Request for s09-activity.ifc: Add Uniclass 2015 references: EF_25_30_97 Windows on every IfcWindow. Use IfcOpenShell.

First a look at what the model holds.

```python
import ifcopenshell

model = ifcopenshell.open("s09-activity.ifc")
print(model.schema)
print("classifications:", [c.Name for c in model.by_type("IfcClassification")])
for ifc_class in ("IfcDoor", "IfcRoof", "IfcStair", "IfcWall", "IfcWindow"):
    print(ifc_class, len(model.by_type(ifc_class)))
```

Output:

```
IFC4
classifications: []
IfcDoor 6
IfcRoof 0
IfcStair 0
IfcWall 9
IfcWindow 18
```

```python
import ifcopenshell
import ifcopenshell.api.classification

model = ifcopenshell.open("s09-activity.ifc")

system = ifcopenshell.api.classification.add_classification(model, classification="Uniclass 2015")

codes = {
    "IfcWindow": ("EF_25_30_97", "Windows"),
}
for ifc_class, (code, name) in codes.items():
    products = model.by_type(ifc_class)
    ifcopenshell.api.classification.add_reference(
        model, products=products, classification=system, identification=code, name=name
    )
    print(code, len(products))

model.write("s09-activity_edited.ifc")
```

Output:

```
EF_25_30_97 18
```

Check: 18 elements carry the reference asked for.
